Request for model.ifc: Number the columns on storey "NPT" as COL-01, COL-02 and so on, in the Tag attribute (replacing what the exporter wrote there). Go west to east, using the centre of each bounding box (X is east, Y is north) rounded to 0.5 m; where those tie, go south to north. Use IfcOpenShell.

First a look at what the model holds.

```python
import ifcopenshell
import ifcopenshell.util.element
import ifcopenshell.util.placement

model = ifcopenshell.open("model.ifc")
print(model.schema)
storey = next(s for s in model.by_type("IfcBuildingStorey") if s.Name == "NPT")
columns = [e for e in ifcopenshell.util.element.get_decomposition(storey) if e.is_a("IfcColumn")]
for e in sorted(columns, key=lambda e: e.id()):
    origin = ifcopenshell.util.placement.get_local_placement(e.ObjectPlacement)[:3, 3]
    print(e.id(), e.Tag, e.Name, origin.round(2) + 0.0, sep=" | ")
```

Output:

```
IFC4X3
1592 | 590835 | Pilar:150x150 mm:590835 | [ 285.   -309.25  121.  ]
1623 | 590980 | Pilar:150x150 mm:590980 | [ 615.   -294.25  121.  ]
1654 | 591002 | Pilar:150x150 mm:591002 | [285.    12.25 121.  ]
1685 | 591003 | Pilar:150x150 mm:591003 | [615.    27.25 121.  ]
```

```python
import ifcopenshell
import ifcopenshell.geom
import ifcopenshell.util.element
import ifcopenshell.util.shape

model = ifcopenshell.open("model.ifc")
settings = ifcopenshell.geom.settings()
settings.set("use-world-coords", True)


def centre(element):
    shape = ifcopenshell.geom.create_shape(settings, element)
    return ifcopenshell.util.shape.get_bbox_centroid(shape.geometry)


storey = next(s for s in model.by_type("IfcBuildingStorey") if s.Name == "NPT")
columns = [e for e in ifcopenshell.util.element.get_decomposition(storey) if e.is_a("IfcColumn")]

# Insertion points can sit at a corner or the storey origin, so sort by the geometry (in metres).
centres = {e: centre(e) for e in columns}
columns.sort(key=lambda e: (round(centres[e][0] / 0.5), centres[e][1]))

for i, e in enumerate(columns, start=1):
    number = f"COL-{i:02d}"
    e.Tag = number
    print(e.id(), number)

model.write("model_updated.ifc")
```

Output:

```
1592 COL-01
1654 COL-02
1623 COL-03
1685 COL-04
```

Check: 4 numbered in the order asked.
